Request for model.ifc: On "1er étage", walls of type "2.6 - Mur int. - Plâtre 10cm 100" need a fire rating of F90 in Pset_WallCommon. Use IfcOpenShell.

First a look at what the model holds.

```python
import ifcopenshell
import ifcopenshell.util.element

model = ifcopenshell.open("model.ifc")
print(model.schema)
storey = next(s for s in model.by_type("IfcBuildingStorey") if s.Name == "1er étage")
walls = [e for e in ifcopenshell.util.element.get_decomposition(storey) if e.is_a("IfcWall")]
seen = {}
for e in walls:
    element_type = ifcopenshell.util.element.get_type(e)
    key = (element_type.Name if element_type != e and element_type else None, ifcopenshell.util.element.get_pset(e, "Pset_WallCommon", "FireRating"))
    seen[key] = seen.get(key, 0) + 1
for (name, value), count in sorted(seen.items(), key=str):
    print(count, "x", name, "|", value)
```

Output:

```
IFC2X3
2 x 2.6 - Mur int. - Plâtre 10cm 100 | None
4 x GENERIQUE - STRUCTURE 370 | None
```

```python
import ifcopenshell
import ifcopenshell.api.pset
import ifcopenshell.util.element

model = ifcopenshell.open("model.ifc")

storey = next(s for s in model.by_type("IfcBuildingStorey") if s.Name == "1er étage")
walls = [e for e in ifcopenshell.util.element.get_decomposition(storey) if e.is_a("IfcWall")]

count = 0
for e in walls:
    element_type = ifcopenshell.util.element.get_type(e)
    if element_type in (None, e) or element_type.Name != "2.6 - Mur int. - Plâtre 10cm 100":
        continue
    # add_pset returns the element's existing set when there is one.
    pset = ifcopenshell.api.pset.add_pset(model, product=e, name="Pset_WallCommon")
    ifcopenshell.api.pset.edit_pset(model, pset=pset, properties={"FireRating": "F90"})
    count += 1

print(count, "walls updated")

model.write("model-out.ifc")
```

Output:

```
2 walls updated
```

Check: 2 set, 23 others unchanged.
